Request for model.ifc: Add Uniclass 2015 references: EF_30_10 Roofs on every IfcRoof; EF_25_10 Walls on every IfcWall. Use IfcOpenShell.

First a look at what the model holds.

```python
import ifcopenshell

model = ifcopenshell.open("model.ifc")
print(model.schema)
print("classifications:", [c.Name for c in model.by_type("IfcClassification")])
for ifc_class in ("IfcDoor", "IfcRoof", "IfcStair", "IfcWall", "IfcWindow"):
    print(ifc_class, len(model.by_type(ifc_class)))
```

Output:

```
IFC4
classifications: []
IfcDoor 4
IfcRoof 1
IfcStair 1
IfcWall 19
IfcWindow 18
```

```python
import ifcopenshell
import ifcopenshell.api.classification

model = ifcopenshell.open("model.ifc")

system = ifcopenshell.api.classification.add_classification(model, classification="Uniclass 2015")

codes = {
    "IfcRoof": ("EF_30_10", "Roofs"),
    "IfcWall": ("EF_25_10", "Walls"),
}
for ifc_class, (code, name) in codes.items():
    products = model.by_type(ifc_class)
    ifcopenshell.api.classification.add_reference(
        model, products=products, classification=system, identification=code, name=name
    )
    print(code, len(products))

model.write("model_v2.ifc")
```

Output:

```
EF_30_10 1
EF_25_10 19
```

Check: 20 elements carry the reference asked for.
